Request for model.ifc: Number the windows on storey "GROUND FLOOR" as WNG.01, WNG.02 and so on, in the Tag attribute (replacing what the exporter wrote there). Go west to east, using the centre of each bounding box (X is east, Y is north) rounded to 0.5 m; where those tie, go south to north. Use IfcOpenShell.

First a look at what the model holds.

```python
import ifcopenshell
import ifcopenshell.util.element
import ifcopenshell.util.placement

model = ifcopenshell.open("model.ifc")
print(model.schema)
storey = next(s for s in model.by_type("IfcBuildingStorey") if s.Name == "GROUND FLOOR")
windows = [e for e in ifcopenshell.util.element.get_decomposition(storey) if e.is_a("IfcWindow")]
for e in sorted(windows, key=lambda e: e.id()):
    origin = ifcopenshell.util.placement.get_local_placement(e.ObjectPlacement)[:3, 3]
    print(e.id(), e.Tag, e.Name, origin.round(2) + 0.0, sep=" | ")
```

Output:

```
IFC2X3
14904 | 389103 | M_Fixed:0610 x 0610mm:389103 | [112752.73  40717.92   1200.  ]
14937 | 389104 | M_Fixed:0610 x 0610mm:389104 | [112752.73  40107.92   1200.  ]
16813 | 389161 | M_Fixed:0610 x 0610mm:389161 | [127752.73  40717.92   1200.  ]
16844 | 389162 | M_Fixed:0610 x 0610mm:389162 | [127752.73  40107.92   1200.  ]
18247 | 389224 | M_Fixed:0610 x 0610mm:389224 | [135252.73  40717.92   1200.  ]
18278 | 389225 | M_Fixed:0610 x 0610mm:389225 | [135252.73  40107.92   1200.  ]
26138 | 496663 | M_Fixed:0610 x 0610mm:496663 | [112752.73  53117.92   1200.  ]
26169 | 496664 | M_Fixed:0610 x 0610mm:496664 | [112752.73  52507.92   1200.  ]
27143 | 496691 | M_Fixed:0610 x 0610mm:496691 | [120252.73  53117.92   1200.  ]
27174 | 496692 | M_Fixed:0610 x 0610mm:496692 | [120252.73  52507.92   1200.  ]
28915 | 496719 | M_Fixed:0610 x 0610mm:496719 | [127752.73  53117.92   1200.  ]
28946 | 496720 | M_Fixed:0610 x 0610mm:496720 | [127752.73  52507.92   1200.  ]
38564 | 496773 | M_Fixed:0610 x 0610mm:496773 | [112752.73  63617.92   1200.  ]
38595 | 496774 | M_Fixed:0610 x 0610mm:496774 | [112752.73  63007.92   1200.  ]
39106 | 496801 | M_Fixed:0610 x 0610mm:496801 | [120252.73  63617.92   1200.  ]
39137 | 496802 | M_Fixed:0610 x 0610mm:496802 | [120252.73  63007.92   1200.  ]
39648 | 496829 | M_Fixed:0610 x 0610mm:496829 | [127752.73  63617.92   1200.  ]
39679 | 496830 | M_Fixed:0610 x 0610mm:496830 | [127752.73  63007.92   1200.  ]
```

```python
import ifcopenshell
import ifcopenshell.geom
import ifcopenshell.util.element
import ifcopenshell.util.shape

model = ifcopenshell.open("model.ifc")
settings = ifcopenshell.geom.settings()
settings.set("use-world-coords", True)


def centre(element):
    shape = ifcopenshell.geom.create_shape(settings, element)
    return ifcopenshell.util.shape.get_bbox_centroid(shape.geometry)


storey = next(s for s in model.by_type("IfcBuildingStorey") if s.Name == "GROUND FLOOR")
windows = [e for e in ifcopenshell.util.element.get_decomposition(storey) if e.is_a("IfcWindow")]

# Insertion points can sit at a corner or the storey origin, so sort by the geometry (in metres).
centres = {e: centre(e) for e in windows}
windows.sort(key=lambda e: (round(centres[e][0] / 0.5), centres[e][1]))

for i, e in enumerate(windows, start=1):
    number = f"WNG.{i:02d}"
    e.Tag = number
    print(e.id(), number)

model.write("model_edited.ifc")
```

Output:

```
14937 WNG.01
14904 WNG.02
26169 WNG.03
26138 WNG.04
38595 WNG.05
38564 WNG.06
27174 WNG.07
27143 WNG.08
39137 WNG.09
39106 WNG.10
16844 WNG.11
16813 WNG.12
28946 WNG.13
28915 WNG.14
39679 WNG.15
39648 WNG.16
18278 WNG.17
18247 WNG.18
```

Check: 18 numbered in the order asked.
